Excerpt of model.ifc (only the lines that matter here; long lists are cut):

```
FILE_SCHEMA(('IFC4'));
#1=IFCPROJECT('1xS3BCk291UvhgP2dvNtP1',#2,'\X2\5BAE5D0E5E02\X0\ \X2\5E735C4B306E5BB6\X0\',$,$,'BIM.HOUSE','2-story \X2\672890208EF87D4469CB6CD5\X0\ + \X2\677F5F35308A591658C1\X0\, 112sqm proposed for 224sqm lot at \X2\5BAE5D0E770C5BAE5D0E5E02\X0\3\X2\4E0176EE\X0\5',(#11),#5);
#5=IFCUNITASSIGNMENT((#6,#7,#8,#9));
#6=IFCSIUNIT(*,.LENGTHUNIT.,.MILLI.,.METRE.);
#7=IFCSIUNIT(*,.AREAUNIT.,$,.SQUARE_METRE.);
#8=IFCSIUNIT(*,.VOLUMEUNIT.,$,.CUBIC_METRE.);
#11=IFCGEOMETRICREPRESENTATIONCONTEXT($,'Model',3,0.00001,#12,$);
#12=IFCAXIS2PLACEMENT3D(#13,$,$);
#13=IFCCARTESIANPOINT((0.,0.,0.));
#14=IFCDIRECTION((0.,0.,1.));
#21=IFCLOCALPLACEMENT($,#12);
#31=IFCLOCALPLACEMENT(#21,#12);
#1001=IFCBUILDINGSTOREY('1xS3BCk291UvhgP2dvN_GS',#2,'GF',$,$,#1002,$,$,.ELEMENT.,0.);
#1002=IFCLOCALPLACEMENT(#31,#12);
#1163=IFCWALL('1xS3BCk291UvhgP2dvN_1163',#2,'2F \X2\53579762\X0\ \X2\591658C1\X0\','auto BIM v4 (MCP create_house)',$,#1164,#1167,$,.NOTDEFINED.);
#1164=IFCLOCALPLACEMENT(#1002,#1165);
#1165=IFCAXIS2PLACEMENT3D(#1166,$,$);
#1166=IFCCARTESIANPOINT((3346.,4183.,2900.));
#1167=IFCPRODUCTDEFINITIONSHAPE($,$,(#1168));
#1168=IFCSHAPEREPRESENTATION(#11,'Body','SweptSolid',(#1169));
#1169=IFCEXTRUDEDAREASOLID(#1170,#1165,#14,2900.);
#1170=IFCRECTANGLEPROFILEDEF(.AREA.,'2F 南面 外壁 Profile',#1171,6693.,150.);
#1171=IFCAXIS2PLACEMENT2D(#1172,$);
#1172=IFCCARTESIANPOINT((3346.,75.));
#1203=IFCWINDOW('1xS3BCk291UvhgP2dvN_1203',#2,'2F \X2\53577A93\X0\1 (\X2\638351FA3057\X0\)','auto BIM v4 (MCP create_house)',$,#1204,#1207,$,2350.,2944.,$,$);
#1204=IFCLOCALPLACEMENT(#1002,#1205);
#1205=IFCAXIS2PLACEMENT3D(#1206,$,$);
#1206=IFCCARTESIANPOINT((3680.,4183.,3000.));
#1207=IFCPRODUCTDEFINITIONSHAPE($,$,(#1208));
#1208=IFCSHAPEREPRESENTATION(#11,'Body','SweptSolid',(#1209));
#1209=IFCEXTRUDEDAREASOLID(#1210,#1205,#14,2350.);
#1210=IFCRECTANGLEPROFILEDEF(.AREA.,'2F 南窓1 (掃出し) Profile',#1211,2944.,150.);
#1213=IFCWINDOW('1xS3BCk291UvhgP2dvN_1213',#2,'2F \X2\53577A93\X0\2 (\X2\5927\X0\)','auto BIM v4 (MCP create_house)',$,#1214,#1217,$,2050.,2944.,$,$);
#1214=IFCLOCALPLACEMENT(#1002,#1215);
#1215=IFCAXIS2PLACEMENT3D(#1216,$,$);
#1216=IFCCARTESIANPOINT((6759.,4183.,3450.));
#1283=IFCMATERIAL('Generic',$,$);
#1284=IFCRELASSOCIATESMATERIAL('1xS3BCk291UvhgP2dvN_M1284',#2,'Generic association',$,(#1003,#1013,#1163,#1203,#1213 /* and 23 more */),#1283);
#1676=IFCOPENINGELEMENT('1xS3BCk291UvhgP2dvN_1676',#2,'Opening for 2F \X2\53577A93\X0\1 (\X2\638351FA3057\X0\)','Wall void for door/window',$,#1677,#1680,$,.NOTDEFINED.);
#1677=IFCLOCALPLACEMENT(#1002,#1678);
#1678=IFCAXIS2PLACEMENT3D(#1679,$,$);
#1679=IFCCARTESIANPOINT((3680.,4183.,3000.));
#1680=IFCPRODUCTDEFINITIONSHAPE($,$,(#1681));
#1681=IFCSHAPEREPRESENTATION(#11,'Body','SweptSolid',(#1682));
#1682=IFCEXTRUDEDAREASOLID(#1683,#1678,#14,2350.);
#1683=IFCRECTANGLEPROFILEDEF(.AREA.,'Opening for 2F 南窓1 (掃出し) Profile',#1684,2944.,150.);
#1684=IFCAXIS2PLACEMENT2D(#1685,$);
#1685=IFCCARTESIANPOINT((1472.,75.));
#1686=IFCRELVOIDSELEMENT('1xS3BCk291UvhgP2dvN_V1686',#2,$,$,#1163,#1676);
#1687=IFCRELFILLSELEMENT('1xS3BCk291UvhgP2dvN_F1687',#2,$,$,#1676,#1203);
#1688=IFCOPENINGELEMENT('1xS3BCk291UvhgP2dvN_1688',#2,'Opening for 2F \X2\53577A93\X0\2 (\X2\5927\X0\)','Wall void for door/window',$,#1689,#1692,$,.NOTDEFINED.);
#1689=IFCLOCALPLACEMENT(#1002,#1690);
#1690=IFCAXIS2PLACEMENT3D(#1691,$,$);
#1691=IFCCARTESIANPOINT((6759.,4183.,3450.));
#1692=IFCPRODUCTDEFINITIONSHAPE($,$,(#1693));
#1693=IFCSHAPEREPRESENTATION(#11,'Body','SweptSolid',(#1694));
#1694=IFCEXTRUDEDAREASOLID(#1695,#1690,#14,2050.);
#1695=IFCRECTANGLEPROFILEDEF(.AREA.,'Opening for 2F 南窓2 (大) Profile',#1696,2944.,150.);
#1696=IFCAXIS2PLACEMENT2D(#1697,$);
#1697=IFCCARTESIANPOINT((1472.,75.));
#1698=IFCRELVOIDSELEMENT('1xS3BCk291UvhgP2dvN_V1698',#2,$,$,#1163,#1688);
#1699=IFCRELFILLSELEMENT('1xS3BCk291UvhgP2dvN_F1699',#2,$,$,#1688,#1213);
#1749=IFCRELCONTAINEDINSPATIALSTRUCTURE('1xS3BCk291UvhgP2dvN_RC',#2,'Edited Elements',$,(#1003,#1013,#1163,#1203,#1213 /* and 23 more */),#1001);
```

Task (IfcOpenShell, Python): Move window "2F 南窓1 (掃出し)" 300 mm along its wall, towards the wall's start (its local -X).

```python
import ifcopenshell
import ifcopenshell.api.geometry
import ifcopenshell.util.placement
import ifcopenshell.util.unit

model = ifcopenshell.open("model.ifc")
unit_scale = ifcopenshell.util.unit.calculate_unit_scale(model)

window = model.by_id(1203)
opening = window.FillsVoids[0].RelatingOpeningElement
wall = opening.VoidsElements[0].RelatingBuildingElement

wall_matrix = ifcopenshell.util.placement.get_local_placement(wall.ObjectPlacement)
shift = wall_matrix[:3, 0] * -0.3 / unit_scale
before = ifcopenshell.util.placement.get_local_placement(window.ObjectPlacement)[:3, 3].copy()

# The window is not placed relative to its opening, so move both.
for product in (opening, window):
    matrix = ifcopenshell.util.placement.get_local_placement(product.ObjectPlacement)
    matrix[:3, 3] += shift
    ifcopenshell.api.geometry.edit_object_placement(model, product=product, matrix=matrix, is_si=False)

after = ifcopenshell.util.placement.get_local_placement(window.ObjectPlacement)[:3, 3]
print("window moved by", (after - before).round(3) + 0.0)

model.write("model_edited.ifc")
```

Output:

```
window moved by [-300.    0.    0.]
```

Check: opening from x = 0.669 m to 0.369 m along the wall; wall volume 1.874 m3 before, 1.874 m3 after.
